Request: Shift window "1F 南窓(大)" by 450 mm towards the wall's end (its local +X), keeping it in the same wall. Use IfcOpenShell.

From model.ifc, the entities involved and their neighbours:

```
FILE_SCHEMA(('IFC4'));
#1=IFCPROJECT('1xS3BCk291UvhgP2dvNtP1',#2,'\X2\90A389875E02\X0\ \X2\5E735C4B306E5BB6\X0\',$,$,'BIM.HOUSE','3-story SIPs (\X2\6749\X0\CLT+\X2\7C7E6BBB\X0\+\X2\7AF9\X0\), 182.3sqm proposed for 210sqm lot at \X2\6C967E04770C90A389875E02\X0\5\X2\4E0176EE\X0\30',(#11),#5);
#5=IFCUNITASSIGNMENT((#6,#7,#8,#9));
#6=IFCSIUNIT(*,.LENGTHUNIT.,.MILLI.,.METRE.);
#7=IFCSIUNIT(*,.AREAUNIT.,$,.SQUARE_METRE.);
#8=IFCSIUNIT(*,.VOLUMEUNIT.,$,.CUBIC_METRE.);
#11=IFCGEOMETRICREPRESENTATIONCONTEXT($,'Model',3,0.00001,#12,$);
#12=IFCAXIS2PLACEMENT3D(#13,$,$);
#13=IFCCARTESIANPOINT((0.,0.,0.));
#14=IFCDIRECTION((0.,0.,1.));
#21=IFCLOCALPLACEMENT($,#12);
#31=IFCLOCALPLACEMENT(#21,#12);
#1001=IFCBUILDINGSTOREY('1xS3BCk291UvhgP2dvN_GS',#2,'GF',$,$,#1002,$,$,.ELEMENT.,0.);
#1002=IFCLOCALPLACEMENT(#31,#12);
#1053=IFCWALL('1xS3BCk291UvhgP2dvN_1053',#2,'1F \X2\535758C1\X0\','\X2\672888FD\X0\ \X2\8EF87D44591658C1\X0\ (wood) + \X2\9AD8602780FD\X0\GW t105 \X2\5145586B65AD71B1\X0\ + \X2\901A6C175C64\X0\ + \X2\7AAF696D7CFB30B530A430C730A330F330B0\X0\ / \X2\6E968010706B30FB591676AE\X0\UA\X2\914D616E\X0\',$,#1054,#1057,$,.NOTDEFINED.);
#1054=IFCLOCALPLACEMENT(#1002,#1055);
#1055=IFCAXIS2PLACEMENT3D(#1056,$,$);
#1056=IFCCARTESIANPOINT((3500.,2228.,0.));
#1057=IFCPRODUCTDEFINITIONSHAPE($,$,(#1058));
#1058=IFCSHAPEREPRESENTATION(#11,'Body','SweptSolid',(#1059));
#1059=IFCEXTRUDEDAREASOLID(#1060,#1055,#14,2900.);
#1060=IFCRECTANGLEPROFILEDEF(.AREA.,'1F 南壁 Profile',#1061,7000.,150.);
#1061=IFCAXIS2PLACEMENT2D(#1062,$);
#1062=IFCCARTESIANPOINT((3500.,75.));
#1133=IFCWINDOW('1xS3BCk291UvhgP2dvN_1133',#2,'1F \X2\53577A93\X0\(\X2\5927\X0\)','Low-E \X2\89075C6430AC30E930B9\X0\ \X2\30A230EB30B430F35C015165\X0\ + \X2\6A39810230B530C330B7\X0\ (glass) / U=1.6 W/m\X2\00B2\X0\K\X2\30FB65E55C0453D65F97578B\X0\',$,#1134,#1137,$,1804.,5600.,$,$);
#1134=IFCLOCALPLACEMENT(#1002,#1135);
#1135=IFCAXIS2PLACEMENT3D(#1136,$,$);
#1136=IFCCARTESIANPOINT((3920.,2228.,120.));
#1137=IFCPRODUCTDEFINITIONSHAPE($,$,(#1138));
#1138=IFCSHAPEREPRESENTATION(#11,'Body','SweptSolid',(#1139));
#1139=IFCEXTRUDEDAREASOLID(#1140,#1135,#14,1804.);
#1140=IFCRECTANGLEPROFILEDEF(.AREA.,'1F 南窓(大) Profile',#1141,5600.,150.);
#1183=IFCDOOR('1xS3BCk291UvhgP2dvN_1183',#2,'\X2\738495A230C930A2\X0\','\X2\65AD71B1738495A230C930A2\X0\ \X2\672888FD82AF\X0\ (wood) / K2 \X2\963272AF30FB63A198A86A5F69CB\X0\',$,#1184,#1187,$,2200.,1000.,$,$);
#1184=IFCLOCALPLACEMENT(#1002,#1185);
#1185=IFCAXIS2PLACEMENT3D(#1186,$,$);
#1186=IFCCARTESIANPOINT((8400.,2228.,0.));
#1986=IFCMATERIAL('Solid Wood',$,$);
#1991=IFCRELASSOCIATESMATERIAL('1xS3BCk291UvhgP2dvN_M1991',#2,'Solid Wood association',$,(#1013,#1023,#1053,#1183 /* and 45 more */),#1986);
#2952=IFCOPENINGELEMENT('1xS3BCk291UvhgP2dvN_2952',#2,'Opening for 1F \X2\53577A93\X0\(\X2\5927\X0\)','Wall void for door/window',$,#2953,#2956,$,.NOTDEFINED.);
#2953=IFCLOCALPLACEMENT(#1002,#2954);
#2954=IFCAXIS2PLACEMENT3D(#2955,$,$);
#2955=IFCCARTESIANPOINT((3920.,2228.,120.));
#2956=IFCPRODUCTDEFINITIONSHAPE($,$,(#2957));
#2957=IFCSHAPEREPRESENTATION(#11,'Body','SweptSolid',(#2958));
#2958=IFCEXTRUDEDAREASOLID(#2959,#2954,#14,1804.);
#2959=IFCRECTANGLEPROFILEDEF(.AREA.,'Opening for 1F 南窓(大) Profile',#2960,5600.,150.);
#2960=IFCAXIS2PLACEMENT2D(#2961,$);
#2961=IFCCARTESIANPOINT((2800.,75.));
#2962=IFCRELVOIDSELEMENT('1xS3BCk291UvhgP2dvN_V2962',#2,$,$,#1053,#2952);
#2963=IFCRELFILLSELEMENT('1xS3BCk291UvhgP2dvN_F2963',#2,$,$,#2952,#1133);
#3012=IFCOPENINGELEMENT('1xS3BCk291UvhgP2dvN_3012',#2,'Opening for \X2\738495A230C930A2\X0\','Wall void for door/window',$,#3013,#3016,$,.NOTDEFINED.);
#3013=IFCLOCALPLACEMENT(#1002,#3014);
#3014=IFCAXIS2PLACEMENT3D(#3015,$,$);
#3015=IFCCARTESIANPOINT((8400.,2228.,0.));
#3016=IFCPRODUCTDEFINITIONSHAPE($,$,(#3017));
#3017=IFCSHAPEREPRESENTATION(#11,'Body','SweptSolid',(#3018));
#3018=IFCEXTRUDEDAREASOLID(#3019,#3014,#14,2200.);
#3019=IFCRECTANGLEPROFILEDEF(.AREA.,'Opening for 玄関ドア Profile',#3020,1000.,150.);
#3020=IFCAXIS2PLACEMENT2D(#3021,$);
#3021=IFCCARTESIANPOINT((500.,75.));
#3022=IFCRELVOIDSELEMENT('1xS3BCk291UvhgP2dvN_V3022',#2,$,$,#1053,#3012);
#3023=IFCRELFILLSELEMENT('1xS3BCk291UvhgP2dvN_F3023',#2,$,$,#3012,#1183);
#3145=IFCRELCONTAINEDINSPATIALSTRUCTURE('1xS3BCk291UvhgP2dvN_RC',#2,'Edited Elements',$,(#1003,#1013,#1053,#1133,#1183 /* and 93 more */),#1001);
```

```python
import ifcopenshell
import ifcopenshell.api.geometry
import ifcopenshell.util.placement
import ifcopenshell.util.unit

model = ifcopenshell.open("model.ifc")
unit_scale = ifcopenshell.util.unit.calculate_unit_scale(model)

window = model.by_guid("1xS3BCk291UvhgP2dvN_1133")
opening = window.FillsVoids[0].RelatingOpeningElement
wall = opening.VoidsElements[0].RelatingBuildingElement

wall_matrix = ifcopenshell.util.placement.get_local_placement(wall.ObjectPlacement)
shift = wall_matrix[:3, 0] * 0.45 / unit_scale
before = ifcopenshell.util.placement.get_local_placement(window.ObjectPlacement)[:3, 3].copy()

# The window is not placed relative to its opening, so move both.
for product in (opening, window):
    matrix = ifcopenshell.util.placement.get_local_placement(product.ObjectPlacement)
    matrix[:3, 3] += shift
    ifcopenshell.api.geometry.edit_object_placement(model, product=product, matrix=matrix, is_si=False)

after = ifcopenshell.util.placement.get_local_placement(window.ObjectPlacement)[:3, 3]
print("window moved by", (after - before).round(3) + 0.0)

model.write("model-out.ifc")
```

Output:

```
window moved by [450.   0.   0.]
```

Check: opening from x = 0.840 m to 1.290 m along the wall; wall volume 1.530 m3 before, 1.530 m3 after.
